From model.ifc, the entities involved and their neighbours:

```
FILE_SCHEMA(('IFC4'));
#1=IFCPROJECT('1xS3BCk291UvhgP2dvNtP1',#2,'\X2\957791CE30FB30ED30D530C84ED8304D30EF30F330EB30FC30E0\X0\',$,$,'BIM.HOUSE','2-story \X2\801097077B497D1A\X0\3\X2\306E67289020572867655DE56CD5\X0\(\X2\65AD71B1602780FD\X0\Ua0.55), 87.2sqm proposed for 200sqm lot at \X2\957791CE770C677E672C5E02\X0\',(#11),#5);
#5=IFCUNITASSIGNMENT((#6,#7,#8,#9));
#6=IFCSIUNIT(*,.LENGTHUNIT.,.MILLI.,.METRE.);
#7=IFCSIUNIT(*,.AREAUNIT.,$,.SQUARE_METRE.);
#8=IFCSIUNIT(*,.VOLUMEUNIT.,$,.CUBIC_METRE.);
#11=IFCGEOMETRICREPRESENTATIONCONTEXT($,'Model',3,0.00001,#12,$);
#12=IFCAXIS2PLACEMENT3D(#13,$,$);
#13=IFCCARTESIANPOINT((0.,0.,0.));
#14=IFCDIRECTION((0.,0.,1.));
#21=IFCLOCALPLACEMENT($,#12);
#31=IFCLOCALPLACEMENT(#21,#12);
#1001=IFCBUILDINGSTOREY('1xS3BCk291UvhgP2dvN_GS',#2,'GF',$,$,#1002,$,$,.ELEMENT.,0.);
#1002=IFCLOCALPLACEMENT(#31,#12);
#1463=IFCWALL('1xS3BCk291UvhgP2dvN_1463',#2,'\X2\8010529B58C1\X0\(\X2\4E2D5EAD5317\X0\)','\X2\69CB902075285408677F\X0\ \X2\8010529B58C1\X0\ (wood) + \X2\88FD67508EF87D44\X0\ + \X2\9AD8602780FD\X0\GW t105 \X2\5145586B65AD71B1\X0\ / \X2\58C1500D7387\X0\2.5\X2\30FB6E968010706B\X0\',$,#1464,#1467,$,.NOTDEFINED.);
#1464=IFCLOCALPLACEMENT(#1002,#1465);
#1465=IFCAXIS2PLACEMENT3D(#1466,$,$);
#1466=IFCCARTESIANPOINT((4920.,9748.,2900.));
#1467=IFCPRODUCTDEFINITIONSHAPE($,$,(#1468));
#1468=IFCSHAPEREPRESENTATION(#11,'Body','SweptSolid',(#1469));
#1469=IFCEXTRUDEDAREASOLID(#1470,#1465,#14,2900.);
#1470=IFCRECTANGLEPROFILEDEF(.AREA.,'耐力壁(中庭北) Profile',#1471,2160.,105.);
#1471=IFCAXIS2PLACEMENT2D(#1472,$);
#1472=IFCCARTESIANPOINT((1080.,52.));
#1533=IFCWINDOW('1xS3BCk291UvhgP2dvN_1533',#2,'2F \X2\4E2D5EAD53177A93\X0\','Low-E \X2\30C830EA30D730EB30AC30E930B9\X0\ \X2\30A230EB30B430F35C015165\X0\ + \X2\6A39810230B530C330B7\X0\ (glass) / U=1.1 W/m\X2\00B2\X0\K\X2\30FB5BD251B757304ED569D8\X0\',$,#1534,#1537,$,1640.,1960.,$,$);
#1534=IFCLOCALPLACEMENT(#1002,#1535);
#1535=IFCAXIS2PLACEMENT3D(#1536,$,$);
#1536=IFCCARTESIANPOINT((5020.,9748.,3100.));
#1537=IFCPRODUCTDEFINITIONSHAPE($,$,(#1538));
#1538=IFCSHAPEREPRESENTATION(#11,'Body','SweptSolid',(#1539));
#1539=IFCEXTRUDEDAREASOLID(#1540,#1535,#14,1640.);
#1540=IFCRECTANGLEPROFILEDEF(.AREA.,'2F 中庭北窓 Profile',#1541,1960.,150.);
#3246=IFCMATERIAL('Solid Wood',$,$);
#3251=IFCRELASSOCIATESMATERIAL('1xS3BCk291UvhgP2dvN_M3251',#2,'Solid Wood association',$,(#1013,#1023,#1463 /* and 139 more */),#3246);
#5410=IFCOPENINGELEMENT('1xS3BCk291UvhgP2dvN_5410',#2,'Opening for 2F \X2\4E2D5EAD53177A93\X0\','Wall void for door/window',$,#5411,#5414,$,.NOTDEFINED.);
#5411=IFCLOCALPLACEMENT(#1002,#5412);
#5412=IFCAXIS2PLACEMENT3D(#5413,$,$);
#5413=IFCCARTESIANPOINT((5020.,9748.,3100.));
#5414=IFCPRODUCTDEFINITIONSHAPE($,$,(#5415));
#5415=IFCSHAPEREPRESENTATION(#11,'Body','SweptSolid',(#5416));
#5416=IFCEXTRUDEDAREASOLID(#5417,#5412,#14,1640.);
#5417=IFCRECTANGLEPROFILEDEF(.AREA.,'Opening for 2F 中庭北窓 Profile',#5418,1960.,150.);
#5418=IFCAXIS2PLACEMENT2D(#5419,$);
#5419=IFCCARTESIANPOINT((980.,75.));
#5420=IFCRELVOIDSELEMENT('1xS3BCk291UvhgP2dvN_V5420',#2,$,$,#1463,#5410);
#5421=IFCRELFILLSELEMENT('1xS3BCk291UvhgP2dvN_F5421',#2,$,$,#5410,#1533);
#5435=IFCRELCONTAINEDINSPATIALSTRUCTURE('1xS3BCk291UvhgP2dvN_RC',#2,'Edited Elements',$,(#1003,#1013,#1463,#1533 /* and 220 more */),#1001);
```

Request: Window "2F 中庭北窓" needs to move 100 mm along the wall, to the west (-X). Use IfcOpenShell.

```python
import ifcopenshell
import ifcopenshell.api.geometry
import ifcopenshell.util.placement
import ifcopenshell.util.unit

model = ifcopenshell.open("model.ifc")
unit_scale = ifcopenshell.util.unit.calculate_unit_scale(model)

window = model.by_guid("1xS3BCk291UvhgP2dvN_1533")
opening = window.FillsVoids[0].RelatingOpeningElement
wall = opening.VoidsElements[0].RelatingBuildingElement

wall_matrix = ifcopenshell.util.placement.get_local_placement(wall.ObjectPlacement)
shift = wall_matrix[:3, 0] * -0.1 / unit_scale
before = ifcopenshell.util.placement.get_local_placement(window.ObjectPlacement)[:3, 3].copy()

# The window is not placed relative to its opening, so move both.
for product in (opening, window):
    matrix = ifcopenshell.util.placement.get_local_placement(product.ObjectPlacement)
    matrix[:3, 3] += shift
    ifcopenshell.api.geometry.edit_object_placement(model, product=product, matrix=matrix, is_si=False)

after = ifcopenshell.util.placement.get_local_placement(window.ObjectPlacement)[:3, 3]
print("window moved by", (after - before).round(3) + 0.0)

model.write("model_updated.ifc")
```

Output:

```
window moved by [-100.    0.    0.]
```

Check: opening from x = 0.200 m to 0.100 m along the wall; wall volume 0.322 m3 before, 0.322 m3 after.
